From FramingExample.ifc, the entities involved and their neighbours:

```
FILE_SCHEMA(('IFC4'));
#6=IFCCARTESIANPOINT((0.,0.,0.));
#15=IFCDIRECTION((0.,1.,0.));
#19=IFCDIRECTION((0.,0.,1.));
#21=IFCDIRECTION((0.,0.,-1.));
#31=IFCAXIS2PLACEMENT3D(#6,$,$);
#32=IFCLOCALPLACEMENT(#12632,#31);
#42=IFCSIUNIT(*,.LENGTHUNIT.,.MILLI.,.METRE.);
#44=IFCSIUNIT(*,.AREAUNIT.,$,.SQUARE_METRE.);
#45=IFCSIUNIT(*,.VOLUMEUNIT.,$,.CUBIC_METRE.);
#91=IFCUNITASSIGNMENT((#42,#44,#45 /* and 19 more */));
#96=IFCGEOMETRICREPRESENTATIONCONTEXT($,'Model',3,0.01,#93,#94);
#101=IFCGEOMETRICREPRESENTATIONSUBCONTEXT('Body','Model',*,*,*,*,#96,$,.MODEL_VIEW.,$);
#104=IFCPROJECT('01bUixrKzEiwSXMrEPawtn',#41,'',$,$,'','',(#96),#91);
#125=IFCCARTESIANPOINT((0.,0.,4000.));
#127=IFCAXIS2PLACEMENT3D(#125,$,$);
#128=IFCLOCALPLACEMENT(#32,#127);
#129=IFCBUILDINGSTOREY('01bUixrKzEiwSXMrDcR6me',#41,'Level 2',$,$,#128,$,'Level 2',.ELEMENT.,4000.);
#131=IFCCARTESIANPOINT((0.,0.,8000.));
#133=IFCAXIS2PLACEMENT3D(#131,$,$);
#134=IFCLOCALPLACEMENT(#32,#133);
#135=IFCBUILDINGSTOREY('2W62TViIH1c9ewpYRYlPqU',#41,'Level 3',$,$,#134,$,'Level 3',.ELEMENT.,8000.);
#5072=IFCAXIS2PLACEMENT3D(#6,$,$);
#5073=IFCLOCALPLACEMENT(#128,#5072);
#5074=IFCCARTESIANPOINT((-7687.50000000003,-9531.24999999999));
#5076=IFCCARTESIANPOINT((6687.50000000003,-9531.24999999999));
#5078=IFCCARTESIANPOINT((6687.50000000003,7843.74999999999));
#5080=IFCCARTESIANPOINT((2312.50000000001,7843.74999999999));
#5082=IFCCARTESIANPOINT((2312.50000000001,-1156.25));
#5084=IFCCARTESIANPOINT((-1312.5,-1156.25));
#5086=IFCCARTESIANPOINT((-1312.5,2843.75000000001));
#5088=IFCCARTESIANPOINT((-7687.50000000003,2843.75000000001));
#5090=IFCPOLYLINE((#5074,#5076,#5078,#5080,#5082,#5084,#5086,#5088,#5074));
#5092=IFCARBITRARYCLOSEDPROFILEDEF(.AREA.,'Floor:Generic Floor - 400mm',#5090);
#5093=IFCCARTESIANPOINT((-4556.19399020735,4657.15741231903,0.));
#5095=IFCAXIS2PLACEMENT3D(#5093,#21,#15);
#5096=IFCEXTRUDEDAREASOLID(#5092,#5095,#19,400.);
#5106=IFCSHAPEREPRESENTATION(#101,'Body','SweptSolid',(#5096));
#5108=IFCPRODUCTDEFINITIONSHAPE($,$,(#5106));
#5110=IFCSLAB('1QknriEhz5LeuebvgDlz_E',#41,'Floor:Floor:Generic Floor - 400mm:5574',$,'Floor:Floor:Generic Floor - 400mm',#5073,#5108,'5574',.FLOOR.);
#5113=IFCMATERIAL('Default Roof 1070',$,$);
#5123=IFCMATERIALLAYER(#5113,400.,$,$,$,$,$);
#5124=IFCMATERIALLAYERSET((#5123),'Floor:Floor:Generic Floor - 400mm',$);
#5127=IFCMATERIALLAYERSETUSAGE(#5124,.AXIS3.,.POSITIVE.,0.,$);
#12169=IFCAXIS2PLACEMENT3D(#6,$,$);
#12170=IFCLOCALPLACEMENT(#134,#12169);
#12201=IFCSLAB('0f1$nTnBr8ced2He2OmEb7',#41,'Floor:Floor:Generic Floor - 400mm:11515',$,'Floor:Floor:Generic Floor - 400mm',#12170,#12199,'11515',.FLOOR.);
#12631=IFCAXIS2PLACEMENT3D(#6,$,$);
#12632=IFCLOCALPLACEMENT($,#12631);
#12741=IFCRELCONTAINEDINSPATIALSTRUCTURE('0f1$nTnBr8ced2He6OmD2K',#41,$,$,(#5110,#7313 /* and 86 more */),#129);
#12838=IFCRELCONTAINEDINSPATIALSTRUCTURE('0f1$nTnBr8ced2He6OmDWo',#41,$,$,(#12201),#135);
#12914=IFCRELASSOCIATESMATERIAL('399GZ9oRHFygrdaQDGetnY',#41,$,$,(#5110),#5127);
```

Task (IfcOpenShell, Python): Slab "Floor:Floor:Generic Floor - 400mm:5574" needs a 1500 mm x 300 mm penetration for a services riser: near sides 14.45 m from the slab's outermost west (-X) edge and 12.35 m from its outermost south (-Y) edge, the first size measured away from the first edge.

```python
import numpy as np
import ifcopenshell
import ifcopenshell.api.feature
import ifcopenshell.api.geometry
import ifcopenshell.api.root
import ifcopenshell.geom
import ifcopenshell.util.placement
import ifcopenshell.util.representation
import ifcopenshell.util.shape
import ifcopenshell.util.unit

model = ifcopenshell.open("FramingExample.ifc")
unit_scale = ifcopenshell.util.unit.calculate_unit_scale(model)
settings = ifcopenshell.geom.settings()


def volume(element):
    """Net volume in cubic metres, openings subtracted."""
    shape = ifcopenshell.geom.create_shape(settings, element)
    return ifcopenshell.util.shape.get_volume(shape.geometry)


slab = model.by_guid("1QknriEhz5LeuebvgDlz_E")
before = volume(slab)

# Extent in the slab's own axes, in metres. The edges named are its -X and -Y sides.
slab_shape = ifcopenshell.geom.create_shape(settings, slab)
vertices = ifcopenshell.util.shape.get_vertices(slab_shape.geometry)
x_min, y_min, bottom = vertices.min(axis=0)
top = vertices[:, 2].max()

opening = ifcopenshell.api.root.create_entity(model, ifc_class="IfcOpeningElement", name="Services riser opening", predefined_type="OPENING")
context = ifcopenshell.util.representation.get_context(model, "Model", "Body", "MODEL_VIEW")
width, depth = 1.5, 0.3
outline = [(0.0, 0.0), (width, 0.0), (width, depth), (0.0, depth), (0.0, 0.0)]
# Overshoot both faces by 50 mm so the cut is clean.
shape = ifcopenshell.api.geometry.add_slab_representation(
    model, context=context, depth=top - bottom + 0.1, polyline=outline
)
ifcopenshell.api.geometry.assign_representation(model, product=opening, representation=shape)

matrix = ifcopenshell.util.placement.get_local_placement(slab.ObjectPlacement)
matrix[:, 3] = matrix @ np.append(np.array([x_min + 14.45, y_min + 12.35, bottom - 0.05]) / unit_scale, 1.0)
ifcopenshell.api.geometry.edit_object_placement(model, product=opening, matrix=matrix, is_si=False)
ifcopenshell.api.feature.add_feature(model, feature=opening, element=slab)

after = volume(slab)

print(f"slab volume {before:.3f} -> {after:.3f} m3")

model.write("FramingExample_rev.ifc")
```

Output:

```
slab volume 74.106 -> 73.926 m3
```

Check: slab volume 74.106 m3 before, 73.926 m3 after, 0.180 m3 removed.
